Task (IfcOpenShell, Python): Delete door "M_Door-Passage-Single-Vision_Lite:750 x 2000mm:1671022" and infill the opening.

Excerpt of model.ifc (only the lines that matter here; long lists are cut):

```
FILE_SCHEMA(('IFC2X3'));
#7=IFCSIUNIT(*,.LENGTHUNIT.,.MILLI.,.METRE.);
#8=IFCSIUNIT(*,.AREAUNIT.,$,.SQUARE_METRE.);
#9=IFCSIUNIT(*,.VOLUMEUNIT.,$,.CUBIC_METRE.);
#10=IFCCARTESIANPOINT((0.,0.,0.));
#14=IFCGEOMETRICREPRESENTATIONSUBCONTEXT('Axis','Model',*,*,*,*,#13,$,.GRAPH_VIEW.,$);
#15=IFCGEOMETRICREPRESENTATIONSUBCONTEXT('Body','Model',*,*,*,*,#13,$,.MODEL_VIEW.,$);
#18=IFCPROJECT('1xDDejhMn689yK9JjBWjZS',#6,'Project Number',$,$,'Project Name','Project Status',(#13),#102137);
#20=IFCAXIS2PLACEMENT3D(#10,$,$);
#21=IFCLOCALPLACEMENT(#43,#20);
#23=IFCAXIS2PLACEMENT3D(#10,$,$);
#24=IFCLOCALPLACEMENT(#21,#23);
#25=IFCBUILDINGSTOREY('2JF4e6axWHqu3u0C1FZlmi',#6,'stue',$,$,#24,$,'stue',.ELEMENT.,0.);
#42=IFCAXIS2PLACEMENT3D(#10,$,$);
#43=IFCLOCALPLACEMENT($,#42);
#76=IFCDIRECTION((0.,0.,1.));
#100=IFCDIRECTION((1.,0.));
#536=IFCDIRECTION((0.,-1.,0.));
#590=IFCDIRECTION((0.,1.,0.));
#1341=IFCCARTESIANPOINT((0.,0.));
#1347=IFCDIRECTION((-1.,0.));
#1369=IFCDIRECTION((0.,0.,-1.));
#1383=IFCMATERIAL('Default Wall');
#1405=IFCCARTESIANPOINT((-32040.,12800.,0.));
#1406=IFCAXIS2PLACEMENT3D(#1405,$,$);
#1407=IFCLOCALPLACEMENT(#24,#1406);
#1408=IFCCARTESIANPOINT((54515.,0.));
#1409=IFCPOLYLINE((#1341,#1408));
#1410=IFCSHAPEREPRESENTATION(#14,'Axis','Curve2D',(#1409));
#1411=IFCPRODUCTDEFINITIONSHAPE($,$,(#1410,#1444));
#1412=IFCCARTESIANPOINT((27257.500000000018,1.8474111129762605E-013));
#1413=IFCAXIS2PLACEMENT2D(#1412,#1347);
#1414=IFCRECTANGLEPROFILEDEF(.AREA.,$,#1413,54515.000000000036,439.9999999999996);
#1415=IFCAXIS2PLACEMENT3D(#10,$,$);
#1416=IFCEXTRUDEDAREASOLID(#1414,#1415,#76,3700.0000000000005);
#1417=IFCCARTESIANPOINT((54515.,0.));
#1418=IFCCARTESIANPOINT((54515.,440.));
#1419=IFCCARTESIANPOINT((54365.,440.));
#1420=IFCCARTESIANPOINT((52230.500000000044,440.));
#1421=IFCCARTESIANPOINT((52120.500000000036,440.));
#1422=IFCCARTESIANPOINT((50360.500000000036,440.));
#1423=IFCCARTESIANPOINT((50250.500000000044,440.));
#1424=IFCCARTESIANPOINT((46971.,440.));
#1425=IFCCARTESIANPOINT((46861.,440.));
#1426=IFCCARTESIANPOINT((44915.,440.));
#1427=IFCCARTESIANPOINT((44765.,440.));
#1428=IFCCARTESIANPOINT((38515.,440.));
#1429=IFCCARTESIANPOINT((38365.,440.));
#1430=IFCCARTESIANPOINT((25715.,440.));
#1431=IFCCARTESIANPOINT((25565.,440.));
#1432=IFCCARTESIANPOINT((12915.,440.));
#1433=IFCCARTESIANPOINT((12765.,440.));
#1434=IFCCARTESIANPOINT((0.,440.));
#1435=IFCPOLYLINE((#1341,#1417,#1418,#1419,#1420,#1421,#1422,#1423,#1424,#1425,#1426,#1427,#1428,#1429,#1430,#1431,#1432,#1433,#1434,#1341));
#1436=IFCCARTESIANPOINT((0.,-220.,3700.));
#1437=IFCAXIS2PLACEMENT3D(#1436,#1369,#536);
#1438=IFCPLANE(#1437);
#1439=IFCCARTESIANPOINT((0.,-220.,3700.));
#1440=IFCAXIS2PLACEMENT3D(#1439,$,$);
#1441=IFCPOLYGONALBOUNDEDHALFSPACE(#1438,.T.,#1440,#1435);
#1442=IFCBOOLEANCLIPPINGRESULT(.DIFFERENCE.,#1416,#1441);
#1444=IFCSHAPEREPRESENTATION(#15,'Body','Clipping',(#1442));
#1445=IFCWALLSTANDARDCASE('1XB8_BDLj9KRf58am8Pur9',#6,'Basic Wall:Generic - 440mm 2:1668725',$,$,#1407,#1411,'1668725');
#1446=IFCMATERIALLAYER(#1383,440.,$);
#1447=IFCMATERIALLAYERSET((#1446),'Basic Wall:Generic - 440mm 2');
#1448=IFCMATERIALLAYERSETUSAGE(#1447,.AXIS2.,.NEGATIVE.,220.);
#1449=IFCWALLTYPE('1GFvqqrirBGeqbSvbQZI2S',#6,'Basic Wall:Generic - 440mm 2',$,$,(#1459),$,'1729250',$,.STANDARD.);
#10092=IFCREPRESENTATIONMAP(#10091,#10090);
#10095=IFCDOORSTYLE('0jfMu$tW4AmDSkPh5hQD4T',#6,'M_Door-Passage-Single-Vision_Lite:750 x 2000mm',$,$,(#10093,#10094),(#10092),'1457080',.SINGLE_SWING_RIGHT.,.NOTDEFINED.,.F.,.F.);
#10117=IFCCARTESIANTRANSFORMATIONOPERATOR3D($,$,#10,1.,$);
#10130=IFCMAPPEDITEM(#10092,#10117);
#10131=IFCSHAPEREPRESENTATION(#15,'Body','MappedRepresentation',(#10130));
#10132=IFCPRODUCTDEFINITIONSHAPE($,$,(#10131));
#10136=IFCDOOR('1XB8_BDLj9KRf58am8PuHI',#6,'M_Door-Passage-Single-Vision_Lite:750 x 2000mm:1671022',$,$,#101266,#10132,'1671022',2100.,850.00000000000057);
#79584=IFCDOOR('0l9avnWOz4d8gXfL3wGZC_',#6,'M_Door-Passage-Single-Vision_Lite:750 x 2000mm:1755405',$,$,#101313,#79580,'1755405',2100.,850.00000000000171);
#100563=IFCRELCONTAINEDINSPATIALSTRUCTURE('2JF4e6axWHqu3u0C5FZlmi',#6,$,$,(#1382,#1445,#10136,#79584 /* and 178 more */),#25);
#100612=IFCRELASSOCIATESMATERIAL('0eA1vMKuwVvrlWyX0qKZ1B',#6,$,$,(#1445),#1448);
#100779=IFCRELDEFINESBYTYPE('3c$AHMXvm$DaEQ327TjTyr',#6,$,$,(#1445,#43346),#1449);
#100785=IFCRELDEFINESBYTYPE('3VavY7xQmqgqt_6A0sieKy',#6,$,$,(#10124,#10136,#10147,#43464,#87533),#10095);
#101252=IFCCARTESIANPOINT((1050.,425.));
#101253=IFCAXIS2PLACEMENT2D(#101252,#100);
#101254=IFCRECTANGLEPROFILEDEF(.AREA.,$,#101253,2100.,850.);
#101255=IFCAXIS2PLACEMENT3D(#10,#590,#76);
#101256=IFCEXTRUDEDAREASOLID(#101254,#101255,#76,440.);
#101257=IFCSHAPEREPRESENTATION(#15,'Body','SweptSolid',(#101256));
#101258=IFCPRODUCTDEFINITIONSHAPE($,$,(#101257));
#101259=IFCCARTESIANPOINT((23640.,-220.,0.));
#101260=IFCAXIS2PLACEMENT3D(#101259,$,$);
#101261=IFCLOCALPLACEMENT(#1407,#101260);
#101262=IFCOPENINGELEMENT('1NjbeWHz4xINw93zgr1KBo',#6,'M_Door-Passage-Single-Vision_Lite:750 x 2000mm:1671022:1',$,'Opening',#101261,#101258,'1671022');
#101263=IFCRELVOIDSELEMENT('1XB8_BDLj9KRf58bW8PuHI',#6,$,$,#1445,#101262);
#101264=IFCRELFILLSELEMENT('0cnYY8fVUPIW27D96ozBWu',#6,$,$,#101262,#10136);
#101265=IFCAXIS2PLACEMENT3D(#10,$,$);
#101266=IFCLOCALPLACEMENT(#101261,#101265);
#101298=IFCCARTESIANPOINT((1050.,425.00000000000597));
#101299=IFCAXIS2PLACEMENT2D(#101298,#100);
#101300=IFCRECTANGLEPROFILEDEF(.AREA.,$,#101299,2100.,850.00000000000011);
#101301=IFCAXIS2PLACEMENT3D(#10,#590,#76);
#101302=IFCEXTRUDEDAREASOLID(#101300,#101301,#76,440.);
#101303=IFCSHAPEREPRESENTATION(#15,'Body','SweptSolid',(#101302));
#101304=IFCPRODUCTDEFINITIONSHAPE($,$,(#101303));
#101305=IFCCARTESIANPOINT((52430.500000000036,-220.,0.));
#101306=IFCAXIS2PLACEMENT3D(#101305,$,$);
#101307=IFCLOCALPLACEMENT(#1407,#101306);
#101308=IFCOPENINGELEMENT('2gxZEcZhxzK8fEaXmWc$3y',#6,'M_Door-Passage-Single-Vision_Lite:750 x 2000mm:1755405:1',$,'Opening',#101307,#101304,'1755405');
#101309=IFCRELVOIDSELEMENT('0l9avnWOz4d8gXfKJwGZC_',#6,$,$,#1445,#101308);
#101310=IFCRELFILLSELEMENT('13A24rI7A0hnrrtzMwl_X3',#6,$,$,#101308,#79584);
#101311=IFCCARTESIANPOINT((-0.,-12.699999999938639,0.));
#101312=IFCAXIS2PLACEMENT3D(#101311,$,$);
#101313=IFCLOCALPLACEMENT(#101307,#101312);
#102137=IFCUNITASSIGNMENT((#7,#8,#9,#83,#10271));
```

```python
import ifcopenshell
import ifcopenshell.api.feature
import ifcopenshell.api.root
import ifcopenshell.geom
import ifcopenshell.util.shape

model = ifcopenshell.open("model.ifc")
settings = ifcopenshell.geom.settings()


def volume(element):
    """Net volume in cubic metres, openings subtracted."""
    shape = ifcopenshell.geom.create_shape(settings, element)
    return ifcopenshell.util.shape.get_volume(shape.geometry)


door = model.by_guid("1XB8_BDLj9KRf58am8PuHI")
opening = door.FillsVoids[0].RelatingOpeningElement
wall = opening.VoidsElements[0].RelatingBuildingElement
before = volume(wall)

ifcopenshell.api.root.remove_product(model, product=door)
ifcopenshell.api.feature.remove_feature(model, feature=opening)

after = volume(wall)

print(f"wall volume {before:.3f} -> {after:.3f} m3")

model.write("model_edited.ifc")
```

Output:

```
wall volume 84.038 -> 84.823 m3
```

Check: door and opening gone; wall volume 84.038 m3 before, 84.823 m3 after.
